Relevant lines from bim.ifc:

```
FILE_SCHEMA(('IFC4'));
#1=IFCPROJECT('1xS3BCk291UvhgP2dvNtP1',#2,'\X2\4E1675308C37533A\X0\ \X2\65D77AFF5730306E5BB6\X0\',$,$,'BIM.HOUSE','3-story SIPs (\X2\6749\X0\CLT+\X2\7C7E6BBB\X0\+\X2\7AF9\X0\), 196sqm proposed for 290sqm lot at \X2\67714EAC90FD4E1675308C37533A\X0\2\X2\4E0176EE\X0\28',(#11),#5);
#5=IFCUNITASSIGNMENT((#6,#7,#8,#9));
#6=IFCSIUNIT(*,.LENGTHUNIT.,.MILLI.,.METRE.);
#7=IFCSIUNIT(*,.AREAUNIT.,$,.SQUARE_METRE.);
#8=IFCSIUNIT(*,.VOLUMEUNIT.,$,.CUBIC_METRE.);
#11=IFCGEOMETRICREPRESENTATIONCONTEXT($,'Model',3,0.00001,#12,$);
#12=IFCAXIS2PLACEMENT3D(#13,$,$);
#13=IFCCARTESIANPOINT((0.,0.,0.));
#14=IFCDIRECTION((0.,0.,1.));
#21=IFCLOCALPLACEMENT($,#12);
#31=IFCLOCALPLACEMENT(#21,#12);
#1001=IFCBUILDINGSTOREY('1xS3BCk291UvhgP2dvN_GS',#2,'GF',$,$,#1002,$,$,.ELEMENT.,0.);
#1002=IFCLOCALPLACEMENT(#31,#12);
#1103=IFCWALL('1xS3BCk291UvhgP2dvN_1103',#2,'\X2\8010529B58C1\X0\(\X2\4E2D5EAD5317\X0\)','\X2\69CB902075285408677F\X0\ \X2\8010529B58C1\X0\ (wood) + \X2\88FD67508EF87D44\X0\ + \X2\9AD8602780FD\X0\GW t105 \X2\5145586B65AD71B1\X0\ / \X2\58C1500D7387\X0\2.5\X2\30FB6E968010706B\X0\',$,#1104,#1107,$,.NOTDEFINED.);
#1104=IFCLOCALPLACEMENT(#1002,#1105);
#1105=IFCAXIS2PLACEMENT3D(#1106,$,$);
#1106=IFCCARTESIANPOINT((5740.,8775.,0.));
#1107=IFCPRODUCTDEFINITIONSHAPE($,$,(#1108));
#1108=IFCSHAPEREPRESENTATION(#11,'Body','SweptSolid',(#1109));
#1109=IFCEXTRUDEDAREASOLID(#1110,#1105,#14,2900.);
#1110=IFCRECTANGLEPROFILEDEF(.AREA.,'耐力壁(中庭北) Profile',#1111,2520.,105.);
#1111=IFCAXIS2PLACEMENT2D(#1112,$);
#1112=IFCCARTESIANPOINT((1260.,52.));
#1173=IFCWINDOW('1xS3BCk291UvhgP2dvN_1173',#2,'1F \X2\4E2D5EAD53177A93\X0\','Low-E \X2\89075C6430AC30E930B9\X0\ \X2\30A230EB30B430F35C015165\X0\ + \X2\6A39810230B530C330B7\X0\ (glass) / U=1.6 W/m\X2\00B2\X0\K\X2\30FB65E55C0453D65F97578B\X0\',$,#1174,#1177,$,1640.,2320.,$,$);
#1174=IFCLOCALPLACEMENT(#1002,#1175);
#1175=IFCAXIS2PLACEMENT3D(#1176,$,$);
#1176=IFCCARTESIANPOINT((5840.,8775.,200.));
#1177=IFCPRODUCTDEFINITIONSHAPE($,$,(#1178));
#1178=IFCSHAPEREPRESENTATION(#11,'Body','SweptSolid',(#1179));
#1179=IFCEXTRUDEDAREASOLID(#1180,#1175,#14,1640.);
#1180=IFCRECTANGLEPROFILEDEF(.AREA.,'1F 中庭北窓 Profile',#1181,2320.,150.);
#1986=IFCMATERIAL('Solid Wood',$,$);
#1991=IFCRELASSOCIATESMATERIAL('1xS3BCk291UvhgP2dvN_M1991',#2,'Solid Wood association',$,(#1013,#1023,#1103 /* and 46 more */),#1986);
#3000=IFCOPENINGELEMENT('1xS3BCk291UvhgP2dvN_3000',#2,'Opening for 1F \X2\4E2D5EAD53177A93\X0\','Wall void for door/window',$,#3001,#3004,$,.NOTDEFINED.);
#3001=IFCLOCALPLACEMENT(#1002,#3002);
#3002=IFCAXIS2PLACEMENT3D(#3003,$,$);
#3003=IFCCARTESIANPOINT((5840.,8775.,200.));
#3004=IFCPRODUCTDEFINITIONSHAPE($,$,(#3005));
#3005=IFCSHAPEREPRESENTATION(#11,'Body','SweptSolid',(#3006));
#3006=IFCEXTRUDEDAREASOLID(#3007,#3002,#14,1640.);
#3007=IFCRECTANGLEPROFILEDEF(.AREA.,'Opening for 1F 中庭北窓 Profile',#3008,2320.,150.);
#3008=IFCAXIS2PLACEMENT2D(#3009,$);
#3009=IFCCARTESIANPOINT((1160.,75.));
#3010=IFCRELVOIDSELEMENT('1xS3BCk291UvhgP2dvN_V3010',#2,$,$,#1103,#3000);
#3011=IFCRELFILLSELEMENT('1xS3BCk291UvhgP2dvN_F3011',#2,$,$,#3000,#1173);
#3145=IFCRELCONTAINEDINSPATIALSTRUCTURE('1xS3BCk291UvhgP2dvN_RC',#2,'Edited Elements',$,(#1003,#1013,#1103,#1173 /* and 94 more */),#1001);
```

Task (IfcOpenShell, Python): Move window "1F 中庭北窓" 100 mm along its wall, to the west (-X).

```python
import ifcopenshell
import ifcopenshell.api.geometry
import ifcopenshell.util.placement

model = ifcopenshell.open("bim.ifc")

window = model.by_guid("1xS3BCk291UvhgP2dvN_1173")
opening = window.FillsVoids[0].RelatingOpeningElement
wall = opening.VoidsElements[0].RelatingBuildingElement

wall_matrix = ifcopenshell.util.placement.get_local_placement(wall.ObjectPlacement)
shift = wall_matrix[:3, 0] * -100.0
before = ifcopenshell.util.placement.get_local_placement(window.ObjectPlacement)[:3, 3].copy()

# The window is not placed relative to its opening, so move both.
for product in (opening, window):
    matrix = ifcopenshell.util.placement.get_local_placement(product.ObjectPlacement)
    matrix[:3, 3] += shift
    ifcopenshell.api.geometry.edit_object_placement(model, product=product, matrix=matrix, is_si=False)

after = ifcopenshell.util.placement.get_local_placement(window.ObjectPlacement)[:3, 3]
print("window moved by", (after - before).round(3) + 0.0)

model.write("bim_rev.ifc")
```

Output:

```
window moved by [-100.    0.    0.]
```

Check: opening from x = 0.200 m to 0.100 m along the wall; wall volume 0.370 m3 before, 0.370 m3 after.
